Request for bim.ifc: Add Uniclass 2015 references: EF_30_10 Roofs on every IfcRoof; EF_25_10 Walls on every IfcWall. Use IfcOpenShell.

First a look at what the model holds.

```python
import ifcopenshell

model = ifcopenshell.open("bim.ifc")
print(model.schema)
print("classifications:", [c.Name for c in model.by_type("IfcClassification")])
for ifc_class in ("IfcDoor", "IfcRoof", "IfcStair", "IfcWall", "IfcWindow"):
    print(ifc_class, len(model.by_type(ifc_class)))
```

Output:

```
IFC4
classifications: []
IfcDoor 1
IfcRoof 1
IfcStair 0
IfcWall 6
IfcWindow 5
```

```python
import ifcopenshell
import ifcopenshell.api.classification

model = ifcopenshell.open("bim.ifc")

system = ifcopenshell.api.classification.add_classification(model, classification="Uniclass 2015")

codes = {
    "IfcRoof": ("EF_30_10", "Roofs"),
    "IfcWall": ("EF_25_10", "Walls"),
}
for ifc_class, (code, name) in codes.items():
    products = model.by_type(ifc_class)
    ifcopenshell.api.classification.add_reference(
        model, products=products, classification=system, identification=code, name=name
    )
    print(code, len(products))

model.write("bim-out.ifc")
```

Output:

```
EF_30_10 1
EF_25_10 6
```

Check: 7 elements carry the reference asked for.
